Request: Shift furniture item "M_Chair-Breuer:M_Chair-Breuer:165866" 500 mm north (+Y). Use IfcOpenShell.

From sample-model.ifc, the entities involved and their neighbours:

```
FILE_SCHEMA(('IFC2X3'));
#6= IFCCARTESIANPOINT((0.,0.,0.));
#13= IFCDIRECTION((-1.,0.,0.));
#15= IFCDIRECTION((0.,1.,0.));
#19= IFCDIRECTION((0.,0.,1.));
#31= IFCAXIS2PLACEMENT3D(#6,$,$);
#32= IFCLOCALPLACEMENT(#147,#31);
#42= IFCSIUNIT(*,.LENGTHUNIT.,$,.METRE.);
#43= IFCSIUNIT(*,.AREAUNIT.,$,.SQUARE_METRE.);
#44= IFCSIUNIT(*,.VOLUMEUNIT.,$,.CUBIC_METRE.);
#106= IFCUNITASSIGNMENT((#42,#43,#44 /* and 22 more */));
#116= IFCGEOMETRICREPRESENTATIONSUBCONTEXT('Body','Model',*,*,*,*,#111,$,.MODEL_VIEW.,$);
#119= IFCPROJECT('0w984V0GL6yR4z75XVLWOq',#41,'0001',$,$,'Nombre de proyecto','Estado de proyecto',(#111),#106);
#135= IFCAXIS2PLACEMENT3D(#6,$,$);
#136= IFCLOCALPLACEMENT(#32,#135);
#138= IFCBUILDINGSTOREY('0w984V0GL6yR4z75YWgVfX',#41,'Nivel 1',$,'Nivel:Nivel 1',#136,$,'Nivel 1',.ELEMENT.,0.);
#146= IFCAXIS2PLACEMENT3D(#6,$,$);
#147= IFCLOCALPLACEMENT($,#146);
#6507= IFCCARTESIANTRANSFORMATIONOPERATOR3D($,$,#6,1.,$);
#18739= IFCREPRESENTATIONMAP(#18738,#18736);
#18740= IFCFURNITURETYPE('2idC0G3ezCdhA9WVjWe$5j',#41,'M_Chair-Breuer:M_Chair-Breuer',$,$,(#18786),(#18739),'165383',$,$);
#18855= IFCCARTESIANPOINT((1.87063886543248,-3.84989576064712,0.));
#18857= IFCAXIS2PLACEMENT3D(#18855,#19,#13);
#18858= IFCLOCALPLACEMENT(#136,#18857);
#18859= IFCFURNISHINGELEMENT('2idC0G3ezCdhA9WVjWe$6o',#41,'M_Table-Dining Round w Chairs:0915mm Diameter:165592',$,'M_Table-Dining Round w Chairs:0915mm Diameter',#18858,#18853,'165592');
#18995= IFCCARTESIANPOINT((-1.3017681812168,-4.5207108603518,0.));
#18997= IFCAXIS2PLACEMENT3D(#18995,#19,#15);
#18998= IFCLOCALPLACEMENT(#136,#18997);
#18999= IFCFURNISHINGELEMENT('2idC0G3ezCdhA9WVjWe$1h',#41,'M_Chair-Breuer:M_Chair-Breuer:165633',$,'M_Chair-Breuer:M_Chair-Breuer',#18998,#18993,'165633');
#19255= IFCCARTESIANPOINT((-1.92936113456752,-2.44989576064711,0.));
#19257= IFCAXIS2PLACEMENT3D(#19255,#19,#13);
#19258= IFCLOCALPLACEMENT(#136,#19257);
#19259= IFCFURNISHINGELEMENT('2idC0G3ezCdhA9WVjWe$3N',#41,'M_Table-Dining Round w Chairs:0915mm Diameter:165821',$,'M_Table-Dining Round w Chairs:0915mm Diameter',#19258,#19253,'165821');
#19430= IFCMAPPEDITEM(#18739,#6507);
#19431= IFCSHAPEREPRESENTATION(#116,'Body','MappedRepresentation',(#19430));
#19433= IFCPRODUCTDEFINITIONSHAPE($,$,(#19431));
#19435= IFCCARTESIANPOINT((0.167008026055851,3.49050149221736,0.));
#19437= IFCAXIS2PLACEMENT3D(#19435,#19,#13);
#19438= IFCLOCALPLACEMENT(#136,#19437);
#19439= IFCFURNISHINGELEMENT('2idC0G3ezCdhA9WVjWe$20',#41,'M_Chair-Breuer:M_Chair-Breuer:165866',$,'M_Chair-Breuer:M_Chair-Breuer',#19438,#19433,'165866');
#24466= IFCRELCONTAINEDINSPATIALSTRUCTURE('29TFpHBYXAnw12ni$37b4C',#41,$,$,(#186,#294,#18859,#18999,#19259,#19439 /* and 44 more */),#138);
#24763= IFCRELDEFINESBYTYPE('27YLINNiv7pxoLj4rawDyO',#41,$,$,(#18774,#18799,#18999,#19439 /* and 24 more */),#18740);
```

```python
import ifcopenshell
import ifcopenshell.api.geometry
import ifcopenshell.util.placement
import ifcopenshell.util.unit

model = ifcopenshell.open("sample-model.ifc")
unit_scale = ifcopenshell.util.unit.calculate_unit_scale(model)

item = model.by_guid("2idC0G3ezCdhA9WVjWe$20")
matrix = ifcopenshell.util.placement.get_local_placement(item.ObjectPlacement)
matrix[1, 3] += 0.5 / unit_scale
ifcopenshell.api.geometry.edit_object_placement(model, product=item, matrix=matrix, is_si=False)

print(ifcopenshell.util.placement.get_local_placement(item.ObjectPlacement).round(3) + 0.0)

model.write("sample-model_rev.ifc")
```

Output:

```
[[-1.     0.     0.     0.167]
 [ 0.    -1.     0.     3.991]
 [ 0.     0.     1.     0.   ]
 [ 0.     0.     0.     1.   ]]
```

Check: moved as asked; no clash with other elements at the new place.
